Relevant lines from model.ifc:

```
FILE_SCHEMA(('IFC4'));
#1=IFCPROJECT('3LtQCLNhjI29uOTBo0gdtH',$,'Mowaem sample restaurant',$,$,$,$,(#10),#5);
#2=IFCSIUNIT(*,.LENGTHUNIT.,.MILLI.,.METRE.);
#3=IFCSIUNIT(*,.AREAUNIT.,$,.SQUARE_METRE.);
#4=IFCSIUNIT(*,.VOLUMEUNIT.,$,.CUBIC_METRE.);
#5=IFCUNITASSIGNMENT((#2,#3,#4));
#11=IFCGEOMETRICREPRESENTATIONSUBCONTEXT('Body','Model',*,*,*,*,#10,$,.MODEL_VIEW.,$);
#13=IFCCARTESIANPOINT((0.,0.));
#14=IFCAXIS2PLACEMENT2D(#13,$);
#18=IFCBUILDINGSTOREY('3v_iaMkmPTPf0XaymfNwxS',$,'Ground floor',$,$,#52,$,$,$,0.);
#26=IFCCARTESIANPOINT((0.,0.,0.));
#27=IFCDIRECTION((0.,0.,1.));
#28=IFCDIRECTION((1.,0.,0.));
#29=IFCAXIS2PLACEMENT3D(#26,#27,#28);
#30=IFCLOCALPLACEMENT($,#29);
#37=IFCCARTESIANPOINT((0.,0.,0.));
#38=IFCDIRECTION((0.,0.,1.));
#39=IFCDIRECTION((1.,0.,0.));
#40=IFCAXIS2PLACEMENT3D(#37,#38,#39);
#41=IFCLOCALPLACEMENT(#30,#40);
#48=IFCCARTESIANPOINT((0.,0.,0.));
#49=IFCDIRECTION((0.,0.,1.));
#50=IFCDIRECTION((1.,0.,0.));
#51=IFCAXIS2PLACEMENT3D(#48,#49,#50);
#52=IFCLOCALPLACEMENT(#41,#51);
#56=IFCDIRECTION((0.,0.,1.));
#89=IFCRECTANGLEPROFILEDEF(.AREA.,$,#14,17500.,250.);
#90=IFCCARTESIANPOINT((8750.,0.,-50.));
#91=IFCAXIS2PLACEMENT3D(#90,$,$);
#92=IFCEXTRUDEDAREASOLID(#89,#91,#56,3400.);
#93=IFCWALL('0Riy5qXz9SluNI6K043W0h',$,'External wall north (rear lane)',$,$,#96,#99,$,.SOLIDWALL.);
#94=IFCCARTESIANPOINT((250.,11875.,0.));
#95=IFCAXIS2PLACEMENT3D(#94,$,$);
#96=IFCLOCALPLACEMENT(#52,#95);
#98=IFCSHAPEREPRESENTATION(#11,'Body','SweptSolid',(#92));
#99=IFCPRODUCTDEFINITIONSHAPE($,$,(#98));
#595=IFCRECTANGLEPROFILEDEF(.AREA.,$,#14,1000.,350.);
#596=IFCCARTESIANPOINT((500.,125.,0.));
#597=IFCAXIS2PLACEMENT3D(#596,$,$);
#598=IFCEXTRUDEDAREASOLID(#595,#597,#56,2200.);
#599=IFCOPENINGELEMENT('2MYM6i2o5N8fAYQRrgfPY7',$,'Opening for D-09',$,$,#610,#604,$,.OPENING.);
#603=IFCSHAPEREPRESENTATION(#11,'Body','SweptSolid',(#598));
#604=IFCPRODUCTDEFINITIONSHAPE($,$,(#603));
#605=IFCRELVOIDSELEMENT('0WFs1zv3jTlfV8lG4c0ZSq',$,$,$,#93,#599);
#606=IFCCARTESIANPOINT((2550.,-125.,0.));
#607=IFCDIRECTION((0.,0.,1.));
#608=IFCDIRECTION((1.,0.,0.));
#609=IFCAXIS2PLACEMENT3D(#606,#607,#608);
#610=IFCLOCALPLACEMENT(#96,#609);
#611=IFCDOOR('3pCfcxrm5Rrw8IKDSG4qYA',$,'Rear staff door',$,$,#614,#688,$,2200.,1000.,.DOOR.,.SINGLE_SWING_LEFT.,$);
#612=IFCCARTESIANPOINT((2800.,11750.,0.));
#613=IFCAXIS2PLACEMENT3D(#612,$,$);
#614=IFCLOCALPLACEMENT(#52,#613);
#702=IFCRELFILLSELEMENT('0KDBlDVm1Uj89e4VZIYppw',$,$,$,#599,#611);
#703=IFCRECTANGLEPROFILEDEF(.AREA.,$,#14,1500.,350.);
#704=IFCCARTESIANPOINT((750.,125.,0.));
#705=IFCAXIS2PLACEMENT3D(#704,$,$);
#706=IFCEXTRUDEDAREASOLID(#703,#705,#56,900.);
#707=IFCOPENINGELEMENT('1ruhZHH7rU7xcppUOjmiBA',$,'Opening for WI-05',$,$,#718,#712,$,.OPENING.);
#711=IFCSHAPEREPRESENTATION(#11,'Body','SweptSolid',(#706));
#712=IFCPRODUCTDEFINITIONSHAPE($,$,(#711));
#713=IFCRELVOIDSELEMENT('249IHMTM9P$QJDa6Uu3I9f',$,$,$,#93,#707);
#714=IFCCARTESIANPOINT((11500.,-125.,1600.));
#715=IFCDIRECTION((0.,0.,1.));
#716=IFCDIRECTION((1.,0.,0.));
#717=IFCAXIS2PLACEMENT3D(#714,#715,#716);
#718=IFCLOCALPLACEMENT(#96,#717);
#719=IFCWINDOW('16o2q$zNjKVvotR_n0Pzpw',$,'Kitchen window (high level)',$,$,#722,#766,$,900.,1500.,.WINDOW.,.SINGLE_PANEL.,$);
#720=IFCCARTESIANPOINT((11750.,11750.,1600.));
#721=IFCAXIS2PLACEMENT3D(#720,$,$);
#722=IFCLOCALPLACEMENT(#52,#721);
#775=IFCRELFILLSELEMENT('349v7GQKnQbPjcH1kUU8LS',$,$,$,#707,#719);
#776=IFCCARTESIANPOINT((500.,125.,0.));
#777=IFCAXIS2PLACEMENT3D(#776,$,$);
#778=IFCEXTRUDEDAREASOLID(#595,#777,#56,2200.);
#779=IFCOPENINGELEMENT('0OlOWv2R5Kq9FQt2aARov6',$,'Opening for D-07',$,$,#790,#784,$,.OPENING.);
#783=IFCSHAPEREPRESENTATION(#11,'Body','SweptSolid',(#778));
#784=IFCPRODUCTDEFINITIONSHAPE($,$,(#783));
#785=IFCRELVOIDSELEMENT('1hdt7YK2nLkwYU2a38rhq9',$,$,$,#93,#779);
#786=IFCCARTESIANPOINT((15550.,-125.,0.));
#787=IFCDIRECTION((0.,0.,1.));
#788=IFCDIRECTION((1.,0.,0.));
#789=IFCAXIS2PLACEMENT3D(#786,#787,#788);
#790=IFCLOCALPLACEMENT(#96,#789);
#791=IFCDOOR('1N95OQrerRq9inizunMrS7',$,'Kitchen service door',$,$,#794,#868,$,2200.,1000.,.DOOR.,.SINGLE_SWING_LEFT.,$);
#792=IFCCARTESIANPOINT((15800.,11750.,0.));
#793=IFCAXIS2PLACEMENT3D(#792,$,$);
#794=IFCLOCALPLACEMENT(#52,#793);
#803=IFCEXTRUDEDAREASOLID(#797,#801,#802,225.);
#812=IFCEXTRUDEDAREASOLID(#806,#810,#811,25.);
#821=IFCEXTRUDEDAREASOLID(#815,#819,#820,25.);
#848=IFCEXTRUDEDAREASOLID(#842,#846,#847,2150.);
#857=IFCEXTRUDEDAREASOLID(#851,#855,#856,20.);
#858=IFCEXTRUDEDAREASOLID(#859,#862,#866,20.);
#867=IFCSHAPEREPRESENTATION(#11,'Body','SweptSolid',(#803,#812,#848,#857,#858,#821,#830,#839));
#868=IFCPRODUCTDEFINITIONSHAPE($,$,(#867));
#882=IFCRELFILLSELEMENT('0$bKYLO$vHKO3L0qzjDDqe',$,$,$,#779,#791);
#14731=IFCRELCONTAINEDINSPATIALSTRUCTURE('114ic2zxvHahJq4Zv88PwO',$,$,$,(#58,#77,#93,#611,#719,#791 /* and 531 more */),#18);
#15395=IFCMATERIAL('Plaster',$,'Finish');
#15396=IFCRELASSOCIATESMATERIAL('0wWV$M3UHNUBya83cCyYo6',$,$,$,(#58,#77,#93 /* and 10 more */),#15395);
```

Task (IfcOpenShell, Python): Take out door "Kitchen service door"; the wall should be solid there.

```python
import ifcopenshell
import ifcopenshell.api.feature
import ifcopenshell.api.root
import ifcopenshell.geom
import ifcopenshell.util.shape

model = ifcopenshell.open("model.ifc")
settings = ifcopenshell.geom.settings()


def volume(element):
    """Net volume in cubic metres, openings subtracted."""
    shape = ifcopenshell.geom.create_shape(settings, element)
    return ifcopenshell.util.shape.get_volume(shape.geometry)


door = model.by_id(791)
opening = door.FillsVoids[0].RelatingOpeningElement
wall = opening.VoidsElements[0].RelatingBuildingElement
before = volume(wall)

ifcopenshell.api.root.remove_product(model, product=door)
ifcopenshell.api.feature.remove_feature(model, feature=opening)

after = volume(wall)

print(f"wall volume {before:.3f} -> {after:.3f} m3")

model.write("model_rev.ifc")
```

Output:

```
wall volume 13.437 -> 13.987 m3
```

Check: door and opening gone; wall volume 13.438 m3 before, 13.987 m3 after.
